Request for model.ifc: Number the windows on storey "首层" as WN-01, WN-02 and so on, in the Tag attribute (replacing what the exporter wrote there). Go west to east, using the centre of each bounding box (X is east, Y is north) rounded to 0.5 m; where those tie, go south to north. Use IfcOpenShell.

First a look at what the model holds.

```python
import ifcopenshell
import ifcopenshell.util.element
import ifcopenshell.util.placement

model = ifcopenshell.open("model.ifc")
print(model.schema)
storey = next(s for s in model.by_type("IfcBuildingStorey") if s.Name == "首层")
windows = [e for e in ifcopenshell.util.element.get_decomposition(storey) if e.is_a("IfcWindow")]
for e in sorted(windows, key=lambda e: e.id()):
    origin = ifcopenshell.util.placement.get_local_placement(e.ObjectPlacement)[:3, 3]
    print(e.id(), e.Tag, e.Name, origin.round(2) + 0.0, sep=" | ")
```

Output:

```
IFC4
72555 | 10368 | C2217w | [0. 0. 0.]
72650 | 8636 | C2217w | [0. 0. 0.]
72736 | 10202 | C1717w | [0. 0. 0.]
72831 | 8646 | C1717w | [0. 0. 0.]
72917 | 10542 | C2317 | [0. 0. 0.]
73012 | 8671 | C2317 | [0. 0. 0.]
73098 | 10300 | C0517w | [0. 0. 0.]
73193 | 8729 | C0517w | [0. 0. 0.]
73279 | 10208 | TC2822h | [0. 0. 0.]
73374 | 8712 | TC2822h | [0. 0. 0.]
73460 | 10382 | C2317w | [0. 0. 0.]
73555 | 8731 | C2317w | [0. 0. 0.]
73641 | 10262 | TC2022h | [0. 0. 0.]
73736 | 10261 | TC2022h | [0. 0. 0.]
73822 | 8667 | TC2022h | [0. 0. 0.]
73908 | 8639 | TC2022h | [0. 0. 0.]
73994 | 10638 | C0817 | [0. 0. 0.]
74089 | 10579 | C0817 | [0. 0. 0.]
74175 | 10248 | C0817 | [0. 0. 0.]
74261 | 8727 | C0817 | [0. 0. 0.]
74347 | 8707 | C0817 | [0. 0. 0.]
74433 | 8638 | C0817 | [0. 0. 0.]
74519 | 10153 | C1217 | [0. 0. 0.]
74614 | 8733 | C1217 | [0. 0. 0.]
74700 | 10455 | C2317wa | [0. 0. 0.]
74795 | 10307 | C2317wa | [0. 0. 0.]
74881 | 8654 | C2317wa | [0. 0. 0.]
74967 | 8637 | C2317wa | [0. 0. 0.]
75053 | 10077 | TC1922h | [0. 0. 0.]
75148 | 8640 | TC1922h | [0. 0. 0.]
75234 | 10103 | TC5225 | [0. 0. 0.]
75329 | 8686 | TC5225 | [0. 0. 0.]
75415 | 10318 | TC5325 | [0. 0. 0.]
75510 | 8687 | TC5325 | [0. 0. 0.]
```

```python
import ifcopenshell
import ifcopenshell.geom
import ifcopenshell.util.element
import ifcopenshell.util.shape

model = ifcopenshell.open("model.ifc")
settings = ifcopenshell.geom.settings()
settings.set("use-world-coords", True)


def centre(element):
    shape = ifcopenshell.geom.create_shape(settings, element)
    return ifcopenshell.util.shape.get_bbox_centroid(shape.geometry)


storey = next(s for s in model.by_type("IfcBuildingStorey") if s.Name == "首层")
windows = [e for e in ifcopenshell.util.element.get_decomposition(storey) if e.is_a("IfcWindow")]

# Insertion points can sit at a corner or the storey origin, so sort by the geometry (in metres).
centres = {e: centre(e) for e in windows}
windows.sort(key=lambda e: (round(centres[e][0] / 0.5), centres[e][1]))

for i, e in enumerate(windows, start=1):
    number = f"WN-{i:02d}"
    e.Tag = number
    print(e.id(), number)

model.write("model_v2.ifc")
```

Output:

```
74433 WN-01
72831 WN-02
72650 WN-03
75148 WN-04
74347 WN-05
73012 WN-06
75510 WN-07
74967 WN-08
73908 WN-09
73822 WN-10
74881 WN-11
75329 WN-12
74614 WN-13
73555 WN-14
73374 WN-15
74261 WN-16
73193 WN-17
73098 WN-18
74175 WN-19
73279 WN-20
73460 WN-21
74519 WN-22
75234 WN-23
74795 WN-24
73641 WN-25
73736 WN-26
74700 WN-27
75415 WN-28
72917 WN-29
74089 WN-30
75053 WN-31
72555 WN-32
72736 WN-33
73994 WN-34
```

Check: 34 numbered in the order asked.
